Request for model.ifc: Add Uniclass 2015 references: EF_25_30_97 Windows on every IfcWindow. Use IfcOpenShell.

First a look at what the model holds.

```python
import ifcopenshell

model = ifcopenshell.open("model.ifc")
print(model.schema)
print("classifications:", [c.Name for c in model.by_type("IfcClassification")])
for ifc_class in ("IfcDoor", "IfcRoof", "IfcStair", "IfcWall", "IfcWindow"):
    print(ifc_class, len(model.by_type(ifc_class)))
```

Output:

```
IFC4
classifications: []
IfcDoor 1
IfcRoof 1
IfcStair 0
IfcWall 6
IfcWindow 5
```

```python
import ifcopenshell
import ifcopenshell.api.classification

model = ifcopenshell.open("model.ifc")

system = ifcopenshell.api.classification.add_classification(model, classification="Uniclass 2015")

codes = {
    "IfcWindow": ("EF_25_30_97", "Windows"),
}
for ifc_class, (code, name) in codes.items():
    products = model.by_type(ifc_class)
    ifcopenshell.api.classification.add_reference(
        model, products=products, classification=system, identification=code, name=name
    )
    print(code, len(products))

model.write("model_updated.ifc")
```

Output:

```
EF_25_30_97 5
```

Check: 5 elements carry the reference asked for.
